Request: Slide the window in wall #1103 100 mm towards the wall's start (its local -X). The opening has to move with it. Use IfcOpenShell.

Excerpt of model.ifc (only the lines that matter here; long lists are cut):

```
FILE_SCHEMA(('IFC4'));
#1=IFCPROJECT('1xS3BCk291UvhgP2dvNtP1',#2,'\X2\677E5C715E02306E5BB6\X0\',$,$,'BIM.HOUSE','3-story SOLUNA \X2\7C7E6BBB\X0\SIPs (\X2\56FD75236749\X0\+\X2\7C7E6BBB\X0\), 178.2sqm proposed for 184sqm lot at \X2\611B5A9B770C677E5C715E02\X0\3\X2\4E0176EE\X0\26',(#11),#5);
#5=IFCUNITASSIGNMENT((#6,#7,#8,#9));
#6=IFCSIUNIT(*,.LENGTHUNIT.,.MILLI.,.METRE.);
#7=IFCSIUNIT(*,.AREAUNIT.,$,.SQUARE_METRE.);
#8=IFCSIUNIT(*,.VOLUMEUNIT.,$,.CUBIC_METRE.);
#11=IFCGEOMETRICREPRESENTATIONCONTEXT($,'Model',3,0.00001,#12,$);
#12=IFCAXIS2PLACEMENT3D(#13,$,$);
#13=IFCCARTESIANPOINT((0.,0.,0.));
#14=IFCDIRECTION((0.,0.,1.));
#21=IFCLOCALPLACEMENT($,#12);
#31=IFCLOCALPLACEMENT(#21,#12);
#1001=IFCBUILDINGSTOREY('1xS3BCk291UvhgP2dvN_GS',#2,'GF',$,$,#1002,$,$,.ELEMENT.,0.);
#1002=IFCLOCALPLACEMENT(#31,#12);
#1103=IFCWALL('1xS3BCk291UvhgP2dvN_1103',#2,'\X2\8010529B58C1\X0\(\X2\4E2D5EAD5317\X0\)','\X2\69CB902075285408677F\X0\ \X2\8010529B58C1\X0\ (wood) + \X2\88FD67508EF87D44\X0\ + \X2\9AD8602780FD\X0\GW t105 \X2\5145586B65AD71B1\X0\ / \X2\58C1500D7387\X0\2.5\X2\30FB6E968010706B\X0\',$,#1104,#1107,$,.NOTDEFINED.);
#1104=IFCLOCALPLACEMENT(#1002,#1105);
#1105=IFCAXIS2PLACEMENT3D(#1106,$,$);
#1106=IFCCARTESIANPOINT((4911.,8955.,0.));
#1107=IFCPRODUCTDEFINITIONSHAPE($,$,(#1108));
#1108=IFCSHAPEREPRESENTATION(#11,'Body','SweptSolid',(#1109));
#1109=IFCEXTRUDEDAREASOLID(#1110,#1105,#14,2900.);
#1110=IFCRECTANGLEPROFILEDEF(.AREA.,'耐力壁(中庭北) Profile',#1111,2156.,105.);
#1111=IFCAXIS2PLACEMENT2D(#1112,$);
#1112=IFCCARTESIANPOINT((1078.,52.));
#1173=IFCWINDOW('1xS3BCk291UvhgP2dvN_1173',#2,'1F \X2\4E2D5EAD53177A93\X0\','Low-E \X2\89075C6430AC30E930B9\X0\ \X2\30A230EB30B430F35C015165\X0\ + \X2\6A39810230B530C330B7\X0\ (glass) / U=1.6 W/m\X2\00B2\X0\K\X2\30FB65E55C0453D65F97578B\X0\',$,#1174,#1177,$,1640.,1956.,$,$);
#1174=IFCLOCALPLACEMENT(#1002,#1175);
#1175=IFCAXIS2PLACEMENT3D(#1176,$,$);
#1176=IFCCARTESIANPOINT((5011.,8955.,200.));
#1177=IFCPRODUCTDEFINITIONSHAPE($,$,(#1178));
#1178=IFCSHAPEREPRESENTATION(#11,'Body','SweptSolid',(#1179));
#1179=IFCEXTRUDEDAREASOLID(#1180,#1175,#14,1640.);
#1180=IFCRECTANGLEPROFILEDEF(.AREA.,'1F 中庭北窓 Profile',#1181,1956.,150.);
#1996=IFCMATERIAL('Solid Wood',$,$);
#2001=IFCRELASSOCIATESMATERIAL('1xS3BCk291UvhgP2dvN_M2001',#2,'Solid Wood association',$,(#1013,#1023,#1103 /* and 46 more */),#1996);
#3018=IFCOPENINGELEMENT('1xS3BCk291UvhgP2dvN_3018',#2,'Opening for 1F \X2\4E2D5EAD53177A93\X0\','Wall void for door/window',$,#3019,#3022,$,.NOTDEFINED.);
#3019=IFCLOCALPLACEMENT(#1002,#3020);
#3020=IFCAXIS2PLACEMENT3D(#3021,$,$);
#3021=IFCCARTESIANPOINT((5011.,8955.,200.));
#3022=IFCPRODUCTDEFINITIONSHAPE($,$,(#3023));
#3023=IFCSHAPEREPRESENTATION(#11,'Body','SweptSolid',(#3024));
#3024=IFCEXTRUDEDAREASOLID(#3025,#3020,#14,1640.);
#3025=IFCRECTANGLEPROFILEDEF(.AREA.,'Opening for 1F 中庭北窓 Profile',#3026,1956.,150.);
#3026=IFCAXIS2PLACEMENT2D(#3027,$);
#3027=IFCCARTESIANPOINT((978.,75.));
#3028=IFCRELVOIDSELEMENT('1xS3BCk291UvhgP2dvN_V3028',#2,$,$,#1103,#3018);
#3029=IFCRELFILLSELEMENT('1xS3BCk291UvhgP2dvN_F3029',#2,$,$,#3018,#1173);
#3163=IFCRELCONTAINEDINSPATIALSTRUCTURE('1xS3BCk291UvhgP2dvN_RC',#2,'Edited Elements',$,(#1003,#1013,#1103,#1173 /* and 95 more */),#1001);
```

```python
import ifcopenshell
import ifcopenshell.api.geometry
import ifcopenshell.util.placement

model = ifcopenshell.open("model.ifc")

window = model.by_guid("1xS3BCk291UvhgP2dvN_1173")
opening = window.FillsVoids[0].RelatingOpeningElement
wall = opening.VoidsElements[0].RelatingBuildingElement

wall_matrix = ifcopenshell.util.placement.get_local_placement(wall.ObjectPlacement)
shift = wall_matrix[:3, 0] * -100.0
before = ifcopenshell.util.placement.get_local_placement(window.ObjectPlacement)[:3, 3].copy()

# The window is not placed relative to its opening, so move both.
for product in (opening, window):
    matrix = ifcopenshell.util.placement.get_local_placement(product.ObjectPlacement)
    matrix[:3, 3] += shift
    ifcopenshell.api.geometry.edit_object_placement(model, product=product, matrix=matrix, is_si=False)

after = ifcopenshell.util.placement.get_local_placement(window.ObjectPlacement)[:3, 3]
print("window moved by", (after - before).round(3) + 0.0)

model.write("model_v2.ifc")
```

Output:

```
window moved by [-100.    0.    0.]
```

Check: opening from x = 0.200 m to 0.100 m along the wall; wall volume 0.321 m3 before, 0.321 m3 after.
